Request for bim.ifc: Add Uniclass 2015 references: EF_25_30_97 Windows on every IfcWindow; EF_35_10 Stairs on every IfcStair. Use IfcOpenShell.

First a look at what the model holds.

```python
import ifcopenshell

model = ifcopenshell.open("bim.ifc")
print(model.schema)
print("classifications:", [c.Name for c in model.by_type("IfcClassification")])
for ifc_class in ("IfcDoor", "IfcRoof", "IfcStair", "IfcWall", "IfcWindow"):
    print(ifc_class, len(model.by_type(ifc_class)))
```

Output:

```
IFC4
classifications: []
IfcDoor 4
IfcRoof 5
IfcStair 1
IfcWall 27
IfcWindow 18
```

```python
import ifcopenshell
import ifcopenshell.api.classification

model = ifcopenshell.open("bim.ifc")

system = ifcopenshell.api.classification.add_classification(model, classification="Uniclass 2015")

codes = {
    "IfcWindow": ("EF_25_30_97", "Windows"),
    "IfcStair": ("EF_35_10", "Stairs"),
}
for ifc_class, (code, name) in codes.items():
    products = model.by_type(ifc_class)
    ifcopenshell.api.classification.add_reference(
        model, products=products, classification=system, identification=code, name=name
    )
    print(code, len(products))

model.write("bim-out.ifc")
```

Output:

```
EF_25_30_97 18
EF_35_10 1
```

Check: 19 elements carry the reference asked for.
